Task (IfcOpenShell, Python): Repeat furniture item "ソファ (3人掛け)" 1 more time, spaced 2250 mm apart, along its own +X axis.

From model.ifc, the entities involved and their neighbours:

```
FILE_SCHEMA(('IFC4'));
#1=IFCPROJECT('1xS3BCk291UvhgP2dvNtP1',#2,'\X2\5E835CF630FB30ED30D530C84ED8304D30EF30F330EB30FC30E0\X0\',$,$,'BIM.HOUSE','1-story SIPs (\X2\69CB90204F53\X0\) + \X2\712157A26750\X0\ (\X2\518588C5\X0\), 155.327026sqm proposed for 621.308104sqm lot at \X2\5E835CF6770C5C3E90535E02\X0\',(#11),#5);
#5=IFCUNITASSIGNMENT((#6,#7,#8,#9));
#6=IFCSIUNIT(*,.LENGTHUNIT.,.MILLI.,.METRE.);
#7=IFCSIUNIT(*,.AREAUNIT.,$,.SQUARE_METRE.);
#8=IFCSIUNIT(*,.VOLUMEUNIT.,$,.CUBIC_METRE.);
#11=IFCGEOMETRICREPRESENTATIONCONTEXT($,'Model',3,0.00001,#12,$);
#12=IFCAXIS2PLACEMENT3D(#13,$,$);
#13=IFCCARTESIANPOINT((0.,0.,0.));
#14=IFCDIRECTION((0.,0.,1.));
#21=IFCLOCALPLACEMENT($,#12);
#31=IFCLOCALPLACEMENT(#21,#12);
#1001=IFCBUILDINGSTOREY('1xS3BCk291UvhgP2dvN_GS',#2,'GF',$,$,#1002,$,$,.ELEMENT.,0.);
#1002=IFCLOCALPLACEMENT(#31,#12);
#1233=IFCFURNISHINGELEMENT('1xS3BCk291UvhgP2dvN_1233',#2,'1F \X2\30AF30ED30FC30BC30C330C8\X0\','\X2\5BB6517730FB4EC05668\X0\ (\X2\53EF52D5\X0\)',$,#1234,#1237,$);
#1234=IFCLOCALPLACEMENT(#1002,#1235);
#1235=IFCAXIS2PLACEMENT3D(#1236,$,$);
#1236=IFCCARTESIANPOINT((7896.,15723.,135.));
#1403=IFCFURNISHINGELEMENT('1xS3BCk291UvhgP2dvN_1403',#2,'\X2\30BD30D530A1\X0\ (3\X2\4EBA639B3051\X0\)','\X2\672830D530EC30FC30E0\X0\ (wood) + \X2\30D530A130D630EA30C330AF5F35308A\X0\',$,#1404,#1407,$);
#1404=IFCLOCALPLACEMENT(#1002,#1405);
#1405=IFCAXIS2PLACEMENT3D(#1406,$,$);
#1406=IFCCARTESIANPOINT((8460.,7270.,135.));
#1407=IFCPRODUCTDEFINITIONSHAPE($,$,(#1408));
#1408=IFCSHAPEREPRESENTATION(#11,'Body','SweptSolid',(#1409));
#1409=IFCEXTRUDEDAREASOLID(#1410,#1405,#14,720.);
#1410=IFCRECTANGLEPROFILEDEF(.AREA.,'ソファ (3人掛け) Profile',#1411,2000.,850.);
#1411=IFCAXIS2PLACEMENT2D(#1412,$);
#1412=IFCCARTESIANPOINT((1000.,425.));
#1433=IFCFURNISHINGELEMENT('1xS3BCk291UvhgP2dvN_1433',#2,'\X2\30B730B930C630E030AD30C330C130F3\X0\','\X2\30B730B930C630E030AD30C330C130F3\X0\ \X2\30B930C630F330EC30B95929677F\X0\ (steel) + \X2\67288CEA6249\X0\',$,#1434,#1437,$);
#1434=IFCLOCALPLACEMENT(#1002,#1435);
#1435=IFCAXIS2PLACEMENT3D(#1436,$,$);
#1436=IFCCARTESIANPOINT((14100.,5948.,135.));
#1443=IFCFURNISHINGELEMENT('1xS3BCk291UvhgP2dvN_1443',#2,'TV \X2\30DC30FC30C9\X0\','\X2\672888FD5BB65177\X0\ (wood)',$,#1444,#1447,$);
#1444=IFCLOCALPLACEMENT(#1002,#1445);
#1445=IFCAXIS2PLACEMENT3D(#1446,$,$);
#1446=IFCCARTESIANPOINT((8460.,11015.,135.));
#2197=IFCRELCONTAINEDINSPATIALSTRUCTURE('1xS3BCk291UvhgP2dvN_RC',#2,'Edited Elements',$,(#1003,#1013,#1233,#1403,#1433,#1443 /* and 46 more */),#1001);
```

```python
import ifcopenshell
import ifcopenshell.api.geometry
import ifcopenshell.api.root
import ifcopenshell.util.element
import ifcopenshell.util.placement

model = ifcopenshell.open("model.ifc")


def reuse_history(source, copy):
    """copy_class also copies each property set's owner history, people and application; keep the originals."""
    for rel in copy.IsDefinedBy:
        if rel.is_a("IfcRelDefinesByProperties") and (history := rel.RelatingPropertyDefinition.OwnerHistory):
            rel.RelatingPropertyDefinition.OwnerHistory = source.OwnerHistory
            ifcopenshell.util.element.remove_deep2(model, history)


source = model.by_guid("1xS3BCk291UvhgP2dvN_1403")
base = ifcopenshell.util.placement.get_local_placement(source.ObjectPlacement)
step = base[:3, 0] * 2250.0

for i in range(1, 2):
    copy = ifcopenshell.api.root.copy_class(model, product=source)
    copy.Representation = ifcopenshell.util.element.copy_deep(
        model, source.Representation, exclude=["IfcGeometricRepresentationContext", "IfcRepresentationMap"]
    )
    reuse_history(source, copy)
    matrix = base.copy()
    matrix[:3, 3] += i * step
    print("added at", matrix[:3, 3].round(3) + 0.0)
    ifcopenshell.api.geometry.edit_object_placement(model, product=copy, matrix=matrix, is_si=False)

model.write("model_updated.ifc")
```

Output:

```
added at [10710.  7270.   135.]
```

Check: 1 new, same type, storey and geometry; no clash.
